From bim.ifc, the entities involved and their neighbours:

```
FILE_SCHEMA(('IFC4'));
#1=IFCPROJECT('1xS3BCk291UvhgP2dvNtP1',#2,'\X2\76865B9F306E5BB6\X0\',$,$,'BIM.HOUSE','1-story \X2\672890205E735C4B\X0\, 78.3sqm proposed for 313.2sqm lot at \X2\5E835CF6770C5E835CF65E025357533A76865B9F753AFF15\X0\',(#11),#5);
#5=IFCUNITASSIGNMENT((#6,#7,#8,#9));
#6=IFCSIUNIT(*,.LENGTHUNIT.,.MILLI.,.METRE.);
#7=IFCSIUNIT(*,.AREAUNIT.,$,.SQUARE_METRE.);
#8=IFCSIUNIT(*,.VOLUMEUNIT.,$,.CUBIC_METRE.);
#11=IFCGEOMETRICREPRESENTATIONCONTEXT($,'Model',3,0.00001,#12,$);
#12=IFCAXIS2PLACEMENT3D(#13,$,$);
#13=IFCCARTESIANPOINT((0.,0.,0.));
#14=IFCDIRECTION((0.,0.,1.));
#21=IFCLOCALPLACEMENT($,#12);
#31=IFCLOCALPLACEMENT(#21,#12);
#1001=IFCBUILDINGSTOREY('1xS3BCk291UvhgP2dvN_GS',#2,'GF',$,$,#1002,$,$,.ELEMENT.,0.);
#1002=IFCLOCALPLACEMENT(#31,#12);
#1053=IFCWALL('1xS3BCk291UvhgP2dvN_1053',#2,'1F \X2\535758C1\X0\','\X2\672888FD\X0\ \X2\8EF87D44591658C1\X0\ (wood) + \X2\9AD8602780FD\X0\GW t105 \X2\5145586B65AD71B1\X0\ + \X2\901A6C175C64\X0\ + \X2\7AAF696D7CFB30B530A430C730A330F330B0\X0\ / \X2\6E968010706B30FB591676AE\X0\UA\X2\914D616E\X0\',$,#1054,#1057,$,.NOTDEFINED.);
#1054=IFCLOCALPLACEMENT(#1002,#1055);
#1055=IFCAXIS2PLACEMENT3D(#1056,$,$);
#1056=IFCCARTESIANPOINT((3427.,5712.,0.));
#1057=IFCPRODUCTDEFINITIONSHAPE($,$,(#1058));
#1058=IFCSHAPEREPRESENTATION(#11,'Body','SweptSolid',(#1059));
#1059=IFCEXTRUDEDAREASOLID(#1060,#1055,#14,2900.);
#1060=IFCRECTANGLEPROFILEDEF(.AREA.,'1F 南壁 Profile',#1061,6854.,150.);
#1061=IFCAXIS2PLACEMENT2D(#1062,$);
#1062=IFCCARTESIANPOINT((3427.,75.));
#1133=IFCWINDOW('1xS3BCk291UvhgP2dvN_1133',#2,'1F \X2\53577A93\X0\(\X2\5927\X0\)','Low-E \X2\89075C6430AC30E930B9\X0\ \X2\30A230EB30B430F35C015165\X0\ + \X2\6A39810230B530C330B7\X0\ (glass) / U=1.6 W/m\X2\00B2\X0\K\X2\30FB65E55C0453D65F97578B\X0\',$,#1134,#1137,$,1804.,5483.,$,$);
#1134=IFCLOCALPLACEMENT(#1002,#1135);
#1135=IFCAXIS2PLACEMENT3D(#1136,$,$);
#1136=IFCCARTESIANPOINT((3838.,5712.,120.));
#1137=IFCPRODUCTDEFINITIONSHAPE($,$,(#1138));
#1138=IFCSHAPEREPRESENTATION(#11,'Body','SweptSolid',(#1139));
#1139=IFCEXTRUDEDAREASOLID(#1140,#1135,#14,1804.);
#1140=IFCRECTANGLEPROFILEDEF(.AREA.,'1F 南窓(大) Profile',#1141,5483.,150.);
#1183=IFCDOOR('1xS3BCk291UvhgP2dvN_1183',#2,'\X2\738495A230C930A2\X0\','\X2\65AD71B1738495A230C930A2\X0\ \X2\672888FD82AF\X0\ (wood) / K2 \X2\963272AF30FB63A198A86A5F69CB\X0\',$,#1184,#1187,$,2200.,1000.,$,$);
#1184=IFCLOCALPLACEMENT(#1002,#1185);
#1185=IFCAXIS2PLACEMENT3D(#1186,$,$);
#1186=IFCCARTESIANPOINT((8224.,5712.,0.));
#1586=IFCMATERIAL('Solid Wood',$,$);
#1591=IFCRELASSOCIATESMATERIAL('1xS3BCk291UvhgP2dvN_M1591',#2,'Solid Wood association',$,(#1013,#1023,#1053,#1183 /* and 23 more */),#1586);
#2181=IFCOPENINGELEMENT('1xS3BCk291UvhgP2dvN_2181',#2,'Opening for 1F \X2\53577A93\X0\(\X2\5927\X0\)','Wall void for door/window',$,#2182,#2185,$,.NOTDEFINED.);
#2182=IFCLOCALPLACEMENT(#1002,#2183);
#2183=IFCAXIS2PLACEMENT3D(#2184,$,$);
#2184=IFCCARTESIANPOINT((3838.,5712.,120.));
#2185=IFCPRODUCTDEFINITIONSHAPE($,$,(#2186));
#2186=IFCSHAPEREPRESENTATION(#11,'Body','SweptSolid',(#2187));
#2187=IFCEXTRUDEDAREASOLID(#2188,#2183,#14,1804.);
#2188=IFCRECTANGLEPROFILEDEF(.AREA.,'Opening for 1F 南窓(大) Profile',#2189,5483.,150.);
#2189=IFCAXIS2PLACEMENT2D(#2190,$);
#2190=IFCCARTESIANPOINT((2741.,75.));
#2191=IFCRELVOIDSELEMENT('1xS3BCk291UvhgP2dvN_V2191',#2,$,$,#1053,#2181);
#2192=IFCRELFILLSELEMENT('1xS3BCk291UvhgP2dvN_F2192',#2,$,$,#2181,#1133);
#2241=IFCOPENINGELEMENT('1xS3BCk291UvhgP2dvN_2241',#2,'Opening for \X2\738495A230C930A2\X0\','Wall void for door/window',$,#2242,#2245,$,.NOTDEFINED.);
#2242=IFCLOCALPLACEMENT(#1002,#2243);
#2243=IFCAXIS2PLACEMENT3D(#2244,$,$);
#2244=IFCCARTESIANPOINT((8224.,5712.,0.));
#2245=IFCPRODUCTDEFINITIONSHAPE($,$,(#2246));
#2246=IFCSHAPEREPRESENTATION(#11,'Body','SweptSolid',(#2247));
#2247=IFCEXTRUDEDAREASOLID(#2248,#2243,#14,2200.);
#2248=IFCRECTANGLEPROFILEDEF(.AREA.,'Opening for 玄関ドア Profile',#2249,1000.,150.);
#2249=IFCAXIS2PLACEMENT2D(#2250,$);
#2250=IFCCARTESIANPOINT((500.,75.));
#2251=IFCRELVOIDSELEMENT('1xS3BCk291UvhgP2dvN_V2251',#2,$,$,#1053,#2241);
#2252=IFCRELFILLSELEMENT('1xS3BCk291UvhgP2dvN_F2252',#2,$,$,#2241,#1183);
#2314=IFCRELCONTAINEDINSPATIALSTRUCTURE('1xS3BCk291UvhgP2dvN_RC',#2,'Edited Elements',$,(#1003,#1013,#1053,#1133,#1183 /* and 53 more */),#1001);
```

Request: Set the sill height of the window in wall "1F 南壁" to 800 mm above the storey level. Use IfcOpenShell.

```python
import numpy as np
import ifcopenshell
import ifcopenshell.api.geometry
import ifcopenshell.geom
import ifcopenshell.util.element
import ifcopenshell.util.placement
import ifcopenshell.util.shape
import ifcopenshell.util.unit

model = ifcopenshell.open("bim.ifc")
unit_scale = ifcopenshell.util.unit.calculate_unit_scale(model)

window = model.by_guid("1xS3BCk291UvhgP2dvN_1133")
opening = window.FillsVoids[0].RelatingOpeningElement
storey = ifcopenshell.util.element.get_container(window, ifc_class="IfcBuildingStorey")
level = ifcopenshell.util.placement.get_local_placement(storey.ObjectPlacement)[2, 3]

# The opening's origin need not be at the sill, so measure its lowest point.
shape = ifcopenshell.geom.create_shape(ifcopenshell.geom.settings(), opening)
bottom = ifcopenshell.util.shape.get_shape_bottom_elevation(shape, shape.geometry) / unit_scale
dz = level + 0.8 / unit_scale - bottom

shift = np.array([0.0, 0.0, dz])
# The window is not placed relative to its opening, so move both.
for product in (opening, window):
    matrix = ifcopenshell.util.placement.get_local_placement(product.ObjectPlacement)
    matrix[:3, 3] += shift
    ifcopenshell.api.geometry.edit_object_placement(model, product=product, matrix=matrix, is_si=False)

print(f"moved by {dz * unit_scale:+.3f} m")

model.write("bim_rev.ifc")
```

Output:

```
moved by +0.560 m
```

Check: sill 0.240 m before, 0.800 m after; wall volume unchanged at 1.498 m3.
